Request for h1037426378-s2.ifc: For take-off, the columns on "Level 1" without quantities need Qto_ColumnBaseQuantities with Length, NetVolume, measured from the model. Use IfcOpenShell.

First a look at what the model holds.

```python
import ifcopenshell
import ifcopenshell.util.element
import ifcopenshell.util.unit

model = ifcopenshell.open("h1037426378-s2.ifc")
print(model.schema)
for unit_type in ("LENGTHUNIT", "AREAUNIT", "VOLUMEUNIT"):
    print(unit_type, ifcopenshell.util.unit.calculate_unit_scale(model, unit_type))
storey = next(s for s in model.by_type("IfcBuildingStorey") if s.Name == "Level 1")
columns = [e for e in ifcopenshell.util.element.get_decomposition(storey) if e.is_a("IfcColumn")]
for e in sorted(columns, key=lambda e: e.id()):
    print(e.id(), e.is_a(), e.Name, list(ifcopenshell.util.element.get_psets(e, qtos_only=True)), sep=" | ")
```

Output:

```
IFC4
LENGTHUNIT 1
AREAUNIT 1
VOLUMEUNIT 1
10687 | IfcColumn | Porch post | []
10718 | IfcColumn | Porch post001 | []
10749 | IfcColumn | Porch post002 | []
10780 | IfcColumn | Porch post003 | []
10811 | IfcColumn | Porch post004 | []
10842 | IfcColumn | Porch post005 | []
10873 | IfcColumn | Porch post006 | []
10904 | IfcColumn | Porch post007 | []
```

```python
import ifcopenshell
import ifcopenshell.api.pset
import ifcopenshell.geom
import ifcopenshell.util.element
import ifcopenshell.util.shape
import ifcopenshell.util.unit

model = ifcopenshell.open("h1037426378-s2.ifc")
unit_scale = ifcopenshell.util.unit.calculate_unit_scale(model)
volume_scale = ifcopenshell.util.unit.calculate_unit_scale(model, "VOLUMEUNIT")
settings = ifcopenshell.geom.settings()

storey = next(s for s in model.by_type("IfcBuildingStorey") if s.Name == "Level 1")
columns = [e for e in ifcopenshell.util.element.get_decomposition(storey) if e.is_a("IfcColumn")]

for e in sorted(columns, key=lambda e: e.id()):
    if ifcopenshell.util.element.get_psets(e, qtos_only=True, should_inherit=False):
        continue
    # Geometry comes back in metres, in the element's own axes.
    shape = ifcopenshell.geom.create_shape(settings, e)
    values = {
        "Length": ifcopenshell.util.shape.get_z(shape.geometry) / unit_scale,
        "NetVolume": ifcopenshell.util.shape.get_volume(shape.geometry) / volume_scale,
    }
    qto = ifcopenshell.api.pset.add_qto(model, product=e, name="Qto_ColumnBaseQuantities")
    ifcopenshell.api.pset.edit_qto(model, qto=qto, properties=values)
    print(e.id(), {k: round(v, 3) for k, v in values.items()})

model.write("h1037426378-s2_v2.ifc")
```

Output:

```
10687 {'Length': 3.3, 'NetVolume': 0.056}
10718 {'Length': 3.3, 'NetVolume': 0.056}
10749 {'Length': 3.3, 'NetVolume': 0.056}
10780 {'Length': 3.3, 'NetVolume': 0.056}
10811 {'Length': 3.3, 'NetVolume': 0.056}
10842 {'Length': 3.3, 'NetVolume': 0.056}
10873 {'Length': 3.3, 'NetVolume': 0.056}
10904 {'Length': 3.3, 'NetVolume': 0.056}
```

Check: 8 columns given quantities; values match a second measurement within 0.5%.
